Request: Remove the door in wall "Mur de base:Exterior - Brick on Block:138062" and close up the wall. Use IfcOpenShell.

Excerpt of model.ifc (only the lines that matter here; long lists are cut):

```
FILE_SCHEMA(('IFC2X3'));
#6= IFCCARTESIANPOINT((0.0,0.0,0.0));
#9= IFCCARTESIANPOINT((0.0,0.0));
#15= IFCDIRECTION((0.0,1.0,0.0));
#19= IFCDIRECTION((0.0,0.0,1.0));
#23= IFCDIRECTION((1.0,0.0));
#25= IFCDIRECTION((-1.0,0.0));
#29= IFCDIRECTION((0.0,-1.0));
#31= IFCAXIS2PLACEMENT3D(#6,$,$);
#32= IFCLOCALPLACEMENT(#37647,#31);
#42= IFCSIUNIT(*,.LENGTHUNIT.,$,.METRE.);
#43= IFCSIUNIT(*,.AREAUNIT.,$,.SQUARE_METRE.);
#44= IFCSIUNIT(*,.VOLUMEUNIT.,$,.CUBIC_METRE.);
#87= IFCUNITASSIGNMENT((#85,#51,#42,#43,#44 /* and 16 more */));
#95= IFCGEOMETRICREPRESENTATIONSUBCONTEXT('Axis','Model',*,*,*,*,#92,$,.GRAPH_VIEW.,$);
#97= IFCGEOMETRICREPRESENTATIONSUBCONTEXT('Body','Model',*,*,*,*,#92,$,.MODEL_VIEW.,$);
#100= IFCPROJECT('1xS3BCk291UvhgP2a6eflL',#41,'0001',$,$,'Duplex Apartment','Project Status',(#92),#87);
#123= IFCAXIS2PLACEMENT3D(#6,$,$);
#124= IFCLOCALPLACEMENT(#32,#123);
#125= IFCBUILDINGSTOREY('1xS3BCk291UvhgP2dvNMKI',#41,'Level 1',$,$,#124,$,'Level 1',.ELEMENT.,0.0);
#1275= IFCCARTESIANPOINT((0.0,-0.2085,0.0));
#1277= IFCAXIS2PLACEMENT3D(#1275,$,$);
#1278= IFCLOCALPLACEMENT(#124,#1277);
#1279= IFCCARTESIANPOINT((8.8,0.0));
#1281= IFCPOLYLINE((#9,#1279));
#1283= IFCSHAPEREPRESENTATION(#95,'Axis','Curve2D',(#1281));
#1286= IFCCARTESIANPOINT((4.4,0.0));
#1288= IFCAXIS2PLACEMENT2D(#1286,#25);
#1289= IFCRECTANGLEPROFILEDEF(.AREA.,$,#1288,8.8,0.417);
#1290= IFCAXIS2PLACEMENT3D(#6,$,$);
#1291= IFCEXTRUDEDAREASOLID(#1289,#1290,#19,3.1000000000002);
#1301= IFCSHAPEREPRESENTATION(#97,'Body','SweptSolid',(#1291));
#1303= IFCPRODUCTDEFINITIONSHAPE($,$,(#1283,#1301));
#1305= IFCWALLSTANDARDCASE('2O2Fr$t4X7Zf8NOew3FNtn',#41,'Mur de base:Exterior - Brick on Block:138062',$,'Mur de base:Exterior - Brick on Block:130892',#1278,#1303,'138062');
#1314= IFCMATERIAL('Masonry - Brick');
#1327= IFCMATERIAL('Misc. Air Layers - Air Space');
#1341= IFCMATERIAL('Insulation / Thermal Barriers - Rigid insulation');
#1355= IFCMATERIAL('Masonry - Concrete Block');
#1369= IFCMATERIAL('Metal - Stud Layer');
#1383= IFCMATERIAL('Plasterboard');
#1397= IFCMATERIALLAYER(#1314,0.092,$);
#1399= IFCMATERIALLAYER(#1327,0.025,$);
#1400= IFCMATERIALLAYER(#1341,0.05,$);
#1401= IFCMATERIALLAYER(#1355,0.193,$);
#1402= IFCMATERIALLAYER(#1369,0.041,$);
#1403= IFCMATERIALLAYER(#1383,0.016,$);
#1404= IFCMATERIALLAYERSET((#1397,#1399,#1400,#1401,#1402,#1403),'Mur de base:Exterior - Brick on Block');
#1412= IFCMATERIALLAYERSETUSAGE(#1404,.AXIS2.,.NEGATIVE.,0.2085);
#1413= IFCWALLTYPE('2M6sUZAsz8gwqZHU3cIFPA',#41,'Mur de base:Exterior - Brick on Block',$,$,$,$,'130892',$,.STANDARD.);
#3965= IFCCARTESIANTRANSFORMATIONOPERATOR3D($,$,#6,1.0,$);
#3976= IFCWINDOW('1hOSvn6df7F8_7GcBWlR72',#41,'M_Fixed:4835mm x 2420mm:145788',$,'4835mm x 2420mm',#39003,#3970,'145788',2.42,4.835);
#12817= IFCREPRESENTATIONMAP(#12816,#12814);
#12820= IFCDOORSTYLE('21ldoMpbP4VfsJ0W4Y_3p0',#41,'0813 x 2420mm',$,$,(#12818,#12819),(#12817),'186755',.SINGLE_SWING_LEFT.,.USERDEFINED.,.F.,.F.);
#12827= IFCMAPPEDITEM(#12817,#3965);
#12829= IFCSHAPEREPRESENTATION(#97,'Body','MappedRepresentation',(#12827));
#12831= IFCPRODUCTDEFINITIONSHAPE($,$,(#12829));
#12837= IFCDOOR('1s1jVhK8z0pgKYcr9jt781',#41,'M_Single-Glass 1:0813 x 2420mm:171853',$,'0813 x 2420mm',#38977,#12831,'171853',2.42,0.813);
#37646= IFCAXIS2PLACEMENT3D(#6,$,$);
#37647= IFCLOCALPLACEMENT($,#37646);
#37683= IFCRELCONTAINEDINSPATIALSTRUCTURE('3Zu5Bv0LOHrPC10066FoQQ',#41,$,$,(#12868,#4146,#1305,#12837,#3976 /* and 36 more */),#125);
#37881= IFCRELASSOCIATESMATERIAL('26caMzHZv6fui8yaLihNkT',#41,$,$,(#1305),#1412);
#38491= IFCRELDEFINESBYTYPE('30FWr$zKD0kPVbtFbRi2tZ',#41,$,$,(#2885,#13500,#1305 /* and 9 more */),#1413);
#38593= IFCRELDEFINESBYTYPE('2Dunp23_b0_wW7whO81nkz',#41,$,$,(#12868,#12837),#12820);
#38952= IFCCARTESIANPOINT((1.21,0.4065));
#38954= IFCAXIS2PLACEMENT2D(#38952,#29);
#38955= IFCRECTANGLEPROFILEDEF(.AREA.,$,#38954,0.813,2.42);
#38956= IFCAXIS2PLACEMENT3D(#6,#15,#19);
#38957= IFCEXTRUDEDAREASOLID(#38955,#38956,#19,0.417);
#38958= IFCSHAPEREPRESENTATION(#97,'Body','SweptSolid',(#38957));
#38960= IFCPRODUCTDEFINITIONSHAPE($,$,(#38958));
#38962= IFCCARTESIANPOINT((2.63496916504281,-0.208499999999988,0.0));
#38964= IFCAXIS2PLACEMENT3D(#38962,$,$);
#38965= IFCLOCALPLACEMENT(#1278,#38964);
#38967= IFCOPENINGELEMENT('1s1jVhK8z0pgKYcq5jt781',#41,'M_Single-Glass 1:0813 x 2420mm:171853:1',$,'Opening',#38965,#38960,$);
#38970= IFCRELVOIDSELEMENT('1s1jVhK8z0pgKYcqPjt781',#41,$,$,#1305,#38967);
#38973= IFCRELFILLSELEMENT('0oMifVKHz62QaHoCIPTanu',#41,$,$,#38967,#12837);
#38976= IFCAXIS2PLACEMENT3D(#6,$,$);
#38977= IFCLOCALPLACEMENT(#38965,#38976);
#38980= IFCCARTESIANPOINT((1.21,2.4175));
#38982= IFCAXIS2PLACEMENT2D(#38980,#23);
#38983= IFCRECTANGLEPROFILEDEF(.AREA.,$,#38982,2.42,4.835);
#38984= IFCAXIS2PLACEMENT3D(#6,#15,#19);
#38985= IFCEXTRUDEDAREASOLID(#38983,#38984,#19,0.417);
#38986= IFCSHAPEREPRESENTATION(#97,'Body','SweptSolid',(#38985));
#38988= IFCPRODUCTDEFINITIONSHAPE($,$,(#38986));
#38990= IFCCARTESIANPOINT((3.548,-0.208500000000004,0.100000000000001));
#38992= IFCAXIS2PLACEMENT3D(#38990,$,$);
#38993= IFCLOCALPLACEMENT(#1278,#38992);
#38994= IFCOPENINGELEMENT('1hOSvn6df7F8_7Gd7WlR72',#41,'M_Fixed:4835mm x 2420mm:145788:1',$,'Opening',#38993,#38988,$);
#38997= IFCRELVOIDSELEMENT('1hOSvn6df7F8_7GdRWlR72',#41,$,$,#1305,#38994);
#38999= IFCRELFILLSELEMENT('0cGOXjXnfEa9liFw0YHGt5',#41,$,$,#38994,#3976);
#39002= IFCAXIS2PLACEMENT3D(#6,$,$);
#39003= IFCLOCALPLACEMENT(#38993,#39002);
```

```python
import ifcopenshell
import ifcopenshell.api.feature
import ifcopenshell.api.root
import ifcopenshell.geom
import ifcopenshell.util.shape

model = ifcopenshell.open("model.ifc")
settings = ifcopenshell.geom.settings()


def volume(element):
    """Net volume in cubic metres, openings subtracted."""
    shape = ifcopenshell.geom.create_shape(settings, element)
    return ifcopenshell.util.shape.get_volume(shape.geometry)


door = model.by_guid("1s1jVhK8z0pgKYcr9jt781")
opening = door.FillsVoids[0].RelatingOpeningElement
wall = opening.VoidsElements[0].RelatingBuildingElement
before = volume(wall)

ifcopenshell.api.root.remove_product(model, product=door)
ifcopenshell.api.feature.remove_feature(model, feature=opening)

after = volume(wall)

print(f"wall volume {before:.3f} -> {after:.3f} m3")

model.write("model_rev.ifc")
```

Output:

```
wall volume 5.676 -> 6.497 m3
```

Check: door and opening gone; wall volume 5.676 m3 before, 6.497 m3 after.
